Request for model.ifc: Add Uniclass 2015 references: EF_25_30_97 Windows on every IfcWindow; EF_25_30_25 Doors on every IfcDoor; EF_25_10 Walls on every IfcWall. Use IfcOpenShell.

First a look at what the model holds.

```python
import ifcopenshell

model = ifcopenshell.open("model.ifc")
print(model.schema)
print("classifications:", [c.Name for c in model.by_type("IfcClassification")])
for ifc_class in ("IfcDoor", "IfcRoof", "IfcStair", "IfcWall", "IfcWindow"):
    print(ifc_class, len(model.by_type(ifc_class)))
```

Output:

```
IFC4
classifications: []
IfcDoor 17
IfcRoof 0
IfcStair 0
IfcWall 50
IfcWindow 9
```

```python
import ifcopenshell
import ifcopenshell.api.classification

model = ifcopenshell.open("model.ifc")

system = ifcopenshell.api.classification.add_classification(model, classification="Uniclass 2015")

codes = {
    "IfcWindow": ("EF_25_30_97", "Windows"),
    "IfcDoor": ("EF_25_30_25", "Doors"),
    "IfcWall": ("EF_25_10", "Walls"),
}
for ifc_class, (code, name) in codes.items():
    products = model.by_type(ifc_class)
    ifcopenshell.api.classification.add_reference(
        model, products=products, classification=system, identification=code, name=name
    )
    print(code, len(products))

model.write("model_edited.ifc")
```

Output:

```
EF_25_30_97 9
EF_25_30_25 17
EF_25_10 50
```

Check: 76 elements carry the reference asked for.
